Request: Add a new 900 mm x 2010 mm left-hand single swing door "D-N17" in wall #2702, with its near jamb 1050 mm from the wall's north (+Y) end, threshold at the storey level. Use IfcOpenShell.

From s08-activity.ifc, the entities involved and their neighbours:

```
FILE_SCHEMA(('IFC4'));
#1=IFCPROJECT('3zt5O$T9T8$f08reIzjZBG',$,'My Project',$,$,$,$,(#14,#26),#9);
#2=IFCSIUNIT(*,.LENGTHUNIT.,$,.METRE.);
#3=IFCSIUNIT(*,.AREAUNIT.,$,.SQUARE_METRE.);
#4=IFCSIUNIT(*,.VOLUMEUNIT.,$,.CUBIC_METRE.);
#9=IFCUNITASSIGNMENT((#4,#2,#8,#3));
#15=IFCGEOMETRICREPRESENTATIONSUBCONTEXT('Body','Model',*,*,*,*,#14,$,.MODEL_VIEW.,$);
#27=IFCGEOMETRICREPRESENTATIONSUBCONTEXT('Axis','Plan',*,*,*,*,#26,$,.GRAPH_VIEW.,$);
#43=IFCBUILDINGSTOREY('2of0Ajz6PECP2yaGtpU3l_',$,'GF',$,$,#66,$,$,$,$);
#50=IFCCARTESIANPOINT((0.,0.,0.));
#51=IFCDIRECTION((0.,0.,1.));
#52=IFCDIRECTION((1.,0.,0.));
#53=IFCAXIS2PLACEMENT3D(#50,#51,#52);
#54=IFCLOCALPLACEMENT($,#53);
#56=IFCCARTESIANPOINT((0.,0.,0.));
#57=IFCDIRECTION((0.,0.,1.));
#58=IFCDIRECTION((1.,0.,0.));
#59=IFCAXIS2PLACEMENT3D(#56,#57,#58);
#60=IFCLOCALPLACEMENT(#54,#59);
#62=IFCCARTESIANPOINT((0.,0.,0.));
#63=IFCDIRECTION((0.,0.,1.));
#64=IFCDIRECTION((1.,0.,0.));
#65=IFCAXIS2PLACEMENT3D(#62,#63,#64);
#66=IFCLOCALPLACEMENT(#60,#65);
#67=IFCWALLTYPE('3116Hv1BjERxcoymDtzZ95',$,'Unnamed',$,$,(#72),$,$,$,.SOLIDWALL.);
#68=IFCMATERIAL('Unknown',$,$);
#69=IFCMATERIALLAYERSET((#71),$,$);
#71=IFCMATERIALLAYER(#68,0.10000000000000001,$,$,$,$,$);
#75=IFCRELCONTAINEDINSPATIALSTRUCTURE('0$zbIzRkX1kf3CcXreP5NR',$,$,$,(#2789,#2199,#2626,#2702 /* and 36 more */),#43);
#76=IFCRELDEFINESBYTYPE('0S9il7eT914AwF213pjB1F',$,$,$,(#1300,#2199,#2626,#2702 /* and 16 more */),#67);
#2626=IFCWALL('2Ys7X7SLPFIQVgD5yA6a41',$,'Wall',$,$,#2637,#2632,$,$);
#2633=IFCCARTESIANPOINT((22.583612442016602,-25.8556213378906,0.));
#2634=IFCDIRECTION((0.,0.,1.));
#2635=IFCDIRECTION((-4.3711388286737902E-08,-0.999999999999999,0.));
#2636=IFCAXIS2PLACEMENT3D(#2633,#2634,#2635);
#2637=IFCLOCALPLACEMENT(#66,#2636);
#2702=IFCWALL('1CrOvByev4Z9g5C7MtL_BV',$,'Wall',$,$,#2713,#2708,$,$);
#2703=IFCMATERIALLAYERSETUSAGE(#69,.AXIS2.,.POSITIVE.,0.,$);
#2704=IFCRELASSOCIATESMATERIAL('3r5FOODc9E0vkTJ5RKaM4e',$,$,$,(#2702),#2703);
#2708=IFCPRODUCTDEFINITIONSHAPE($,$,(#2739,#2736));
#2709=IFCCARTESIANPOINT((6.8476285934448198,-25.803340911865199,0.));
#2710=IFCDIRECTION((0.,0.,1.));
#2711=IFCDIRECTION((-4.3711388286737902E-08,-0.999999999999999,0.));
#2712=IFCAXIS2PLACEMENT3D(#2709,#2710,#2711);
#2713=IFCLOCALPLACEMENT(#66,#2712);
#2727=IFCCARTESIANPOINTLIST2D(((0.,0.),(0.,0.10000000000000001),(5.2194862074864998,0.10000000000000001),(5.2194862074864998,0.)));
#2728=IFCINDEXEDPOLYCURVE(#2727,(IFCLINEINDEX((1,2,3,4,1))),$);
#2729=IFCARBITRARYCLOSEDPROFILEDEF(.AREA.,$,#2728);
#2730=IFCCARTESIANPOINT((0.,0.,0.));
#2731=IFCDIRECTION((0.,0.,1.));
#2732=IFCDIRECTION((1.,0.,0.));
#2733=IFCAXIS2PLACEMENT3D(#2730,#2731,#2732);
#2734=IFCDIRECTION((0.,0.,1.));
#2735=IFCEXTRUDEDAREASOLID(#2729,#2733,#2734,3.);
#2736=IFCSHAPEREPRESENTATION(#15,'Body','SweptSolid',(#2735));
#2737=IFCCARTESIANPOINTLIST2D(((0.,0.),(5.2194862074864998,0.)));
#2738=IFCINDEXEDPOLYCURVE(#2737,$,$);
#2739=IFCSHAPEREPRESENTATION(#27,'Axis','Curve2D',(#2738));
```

```python
import numpy as np
import ifcopenshell
import ifcopenshell.api.feature
import ifcopenshell.api.geometry
import ifcopenshell.api.root
import ifcopenshell.api.spatial
import ifcopenshell.geom
import ifcopenshell.util.element
import ifcopenshell.util.placement
import ifcopenshell.util.representation
import ifcopenshell.util.shape
import ifcopenshell.util.unit

model = ifcopenshell.open("s08-activity.ifc")
unit_scale = ifcopenshell.util.unit.calculate_unit_scale(model)
settings = ifcopenshell.geom.settings()


def volume(element):
    """Net volume in cubic metres, openings subtracted."""
    shape = ifcopenshell.geom.create_shape(settings, element)
    return ifcopenshell.util.shape.get_volume(shape.geometry)


wall = model.by_id(2702)
storey = ifcopenshell.util.element.get_container(wall, ifc_class="IfcBuildingStorey")
context = ifcopenshell.util.representation.get_context(model, "Model", "Body", "MODEL_VIEW")
before = volume(wall)

width, height, from_end, sill = 0.9, 2.01, 1.05, 0.0  # metres

# The wall runs along its own X axis, and the end named is its -X end.
wall_shape = ifcopenshell.geom.create_shape(settings, wall)
x, y, z = ifcopenshell.util.shape.get_vertices(wall_shape.geometry).T
start = x.min() + from_end
face, thickness = float(y.min()), float(y.max() - y.min())
wall_matrix = ifcopenshell.util.placement.get_local_placement(wall.ObjectPlacement)
level = ifcopenshell.util.placement.get_local_placement(storey.ObjectPlacement)[2, 3]


def in_wall(x, y):
    """Placement at x, y metres in the wall's axes, at sill height."""
    matrix = wall_matrix.copy()
    matrix[:, 3] = wall_matrix @ np.array([x / unit_scale, y / unit_scale, 0.0, 1.0])
    matrix[2, 3] = level + sill / unit_scale
    return matrix


# Opening: a box that overshoots both wall faces by 50 mm.
opening = ifcopenshell.api.root.create_entity(model, ifc_class="IfcOpeningElement", predefined_type="OPENING")
box = ifcopenshell.api.geometry.add_wall_representation(
    model, context=context, length=width, height=height, thickness=thickness + 0.1
)
ifcopenshell.api.geometry.assign_representation(model, product=opening, representation=box)
ifcopenshell.api.geometry.edit_object_placement(model, product=opening, matrix=in_wall(start, face - 0.05), is_si=False)
ifcopenshell.api.feature.add_feature(model, feature=opening, element=wall)

door = ifcopenshell.api.root.create_entity(model, ifc_class="IfcDoor", name="D-N17", predefined_type="DOOR")
door.OverallWidth, door.OverallHeight = width / unit_scale, height / unit_scale
door.OperationType = "SINGLE_SWING_LEFT"
body = ifcopenshell.api.geometry.add_door_representation(
    model,
    context=context,
    overall_width=door.OverallWidth,
    overall_height=door.OverallHeight,
    operation_type="SINGLE_SWING_LEFT",
    lining_properties={"LiningDepth": thickness / unit_scale, "ThresholdDepth": thickness / unit_scale},
)
ifcopenshell.api.geometry.assign_representation(model, product=door, representation=body)
ifcopenshell.api.spatial.assign_container(model, products=[door], relating_structure=storey)
ifcopenshell.api.feature.add_filling(model, opening=opening, element=door)

# The lining spans the wall, so the door starts at the wall face.
ifcopenshell.api.geometry.edit_object_placement(model, product=door, matrix=in_wall(start, face), is_si=False)

after = volume(wall)

print(f"wall volume {before:.3f} -> {after:.3f} m3")

model.write("s08-activity_rev.ifc")
```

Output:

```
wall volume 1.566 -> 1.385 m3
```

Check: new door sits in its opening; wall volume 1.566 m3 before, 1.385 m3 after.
